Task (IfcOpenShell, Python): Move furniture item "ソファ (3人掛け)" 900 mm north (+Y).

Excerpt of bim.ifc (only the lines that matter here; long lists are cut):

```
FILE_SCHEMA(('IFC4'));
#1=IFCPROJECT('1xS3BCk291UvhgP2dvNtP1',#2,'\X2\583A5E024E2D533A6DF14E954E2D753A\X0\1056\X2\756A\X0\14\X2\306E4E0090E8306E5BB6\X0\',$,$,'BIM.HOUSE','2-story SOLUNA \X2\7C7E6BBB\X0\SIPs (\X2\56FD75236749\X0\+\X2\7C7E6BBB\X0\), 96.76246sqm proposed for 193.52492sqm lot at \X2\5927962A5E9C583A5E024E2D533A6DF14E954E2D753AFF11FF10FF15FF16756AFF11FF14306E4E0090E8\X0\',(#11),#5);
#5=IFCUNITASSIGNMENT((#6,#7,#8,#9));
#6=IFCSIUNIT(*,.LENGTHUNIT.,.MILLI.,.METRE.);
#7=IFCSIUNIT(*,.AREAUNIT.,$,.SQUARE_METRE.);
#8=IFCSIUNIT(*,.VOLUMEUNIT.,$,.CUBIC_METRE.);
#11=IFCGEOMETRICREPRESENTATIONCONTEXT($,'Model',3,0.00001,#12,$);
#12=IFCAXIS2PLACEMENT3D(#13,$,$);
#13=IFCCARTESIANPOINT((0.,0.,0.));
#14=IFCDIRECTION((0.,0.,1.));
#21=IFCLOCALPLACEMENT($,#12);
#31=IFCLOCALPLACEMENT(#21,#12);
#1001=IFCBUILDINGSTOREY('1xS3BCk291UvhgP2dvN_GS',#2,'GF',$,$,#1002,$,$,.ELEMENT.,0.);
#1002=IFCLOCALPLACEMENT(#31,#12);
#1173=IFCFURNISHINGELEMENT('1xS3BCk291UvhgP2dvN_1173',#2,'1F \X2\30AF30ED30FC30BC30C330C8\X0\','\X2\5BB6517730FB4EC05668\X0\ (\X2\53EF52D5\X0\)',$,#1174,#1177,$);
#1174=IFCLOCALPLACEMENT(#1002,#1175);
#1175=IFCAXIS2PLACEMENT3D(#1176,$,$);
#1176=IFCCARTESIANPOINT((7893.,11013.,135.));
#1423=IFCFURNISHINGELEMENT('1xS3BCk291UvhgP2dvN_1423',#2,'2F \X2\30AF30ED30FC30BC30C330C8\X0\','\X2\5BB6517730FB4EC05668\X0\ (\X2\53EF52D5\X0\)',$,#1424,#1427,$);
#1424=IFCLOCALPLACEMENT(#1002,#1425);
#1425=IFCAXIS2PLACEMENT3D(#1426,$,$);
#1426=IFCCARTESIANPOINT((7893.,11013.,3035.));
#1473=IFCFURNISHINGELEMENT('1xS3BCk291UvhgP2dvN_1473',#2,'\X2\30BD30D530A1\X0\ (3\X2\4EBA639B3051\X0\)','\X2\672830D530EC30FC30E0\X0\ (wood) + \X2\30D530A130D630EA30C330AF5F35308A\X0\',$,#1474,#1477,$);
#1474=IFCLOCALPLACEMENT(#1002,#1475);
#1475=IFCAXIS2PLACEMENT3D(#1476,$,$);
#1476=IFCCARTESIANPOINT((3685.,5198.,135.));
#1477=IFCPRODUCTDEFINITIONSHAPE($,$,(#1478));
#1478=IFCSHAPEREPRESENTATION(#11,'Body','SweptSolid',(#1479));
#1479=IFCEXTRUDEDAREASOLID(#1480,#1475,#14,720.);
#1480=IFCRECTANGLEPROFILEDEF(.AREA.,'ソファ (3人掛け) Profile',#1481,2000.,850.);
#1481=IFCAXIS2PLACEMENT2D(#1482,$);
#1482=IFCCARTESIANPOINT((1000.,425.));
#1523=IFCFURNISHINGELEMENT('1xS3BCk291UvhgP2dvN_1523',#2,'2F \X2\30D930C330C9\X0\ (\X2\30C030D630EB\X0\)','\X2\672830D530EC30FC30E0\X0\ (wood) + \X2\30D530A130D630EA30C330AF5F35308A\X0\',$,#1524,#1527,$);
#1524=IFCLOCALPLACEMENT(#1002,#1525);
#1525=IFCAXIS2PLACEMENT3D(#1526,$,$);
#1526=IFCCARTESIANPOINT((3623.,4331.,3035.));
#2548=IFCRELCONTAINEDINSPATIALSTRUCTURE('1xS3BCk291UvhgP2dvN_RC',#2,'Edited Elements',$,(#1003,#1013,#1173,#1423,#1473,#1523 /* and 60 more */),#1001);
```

```python
import ifcopenshell
import ifcopenshell.api.geometry
import ifcopenshell.util.placement
import ifcopenshell.util.unit

model = ifcopenshell.open("bim.ifc")
unit_scale = ifcopenshell.util.unit.calculate_unit_scale(model)

item = model.by_guid("1xS3BCk291UvhgP2dvN_1473")
matrix = ifcopenshell.util.placement.get_local_placement(item.ObjectPlacement)
matrix[1, 3] += 0.9 / unit_scale
ifcopenshell.api.geometry.edit_object_placement(model, product=item, matrix=matrix, is_si=False)

print(ifcopenshell.util.placement.get_local_placement(item.ObjectPlacement).round(3) + 0.0)

model.write("bim_v2.ifc")
```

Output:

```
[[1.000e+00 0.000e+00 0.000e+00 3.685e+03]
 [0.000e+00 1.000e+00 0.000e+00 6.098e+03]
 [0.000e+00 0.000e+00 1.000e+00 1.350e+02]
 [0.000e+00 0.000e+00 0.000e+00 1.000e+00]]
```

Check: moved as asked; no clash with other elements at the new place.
